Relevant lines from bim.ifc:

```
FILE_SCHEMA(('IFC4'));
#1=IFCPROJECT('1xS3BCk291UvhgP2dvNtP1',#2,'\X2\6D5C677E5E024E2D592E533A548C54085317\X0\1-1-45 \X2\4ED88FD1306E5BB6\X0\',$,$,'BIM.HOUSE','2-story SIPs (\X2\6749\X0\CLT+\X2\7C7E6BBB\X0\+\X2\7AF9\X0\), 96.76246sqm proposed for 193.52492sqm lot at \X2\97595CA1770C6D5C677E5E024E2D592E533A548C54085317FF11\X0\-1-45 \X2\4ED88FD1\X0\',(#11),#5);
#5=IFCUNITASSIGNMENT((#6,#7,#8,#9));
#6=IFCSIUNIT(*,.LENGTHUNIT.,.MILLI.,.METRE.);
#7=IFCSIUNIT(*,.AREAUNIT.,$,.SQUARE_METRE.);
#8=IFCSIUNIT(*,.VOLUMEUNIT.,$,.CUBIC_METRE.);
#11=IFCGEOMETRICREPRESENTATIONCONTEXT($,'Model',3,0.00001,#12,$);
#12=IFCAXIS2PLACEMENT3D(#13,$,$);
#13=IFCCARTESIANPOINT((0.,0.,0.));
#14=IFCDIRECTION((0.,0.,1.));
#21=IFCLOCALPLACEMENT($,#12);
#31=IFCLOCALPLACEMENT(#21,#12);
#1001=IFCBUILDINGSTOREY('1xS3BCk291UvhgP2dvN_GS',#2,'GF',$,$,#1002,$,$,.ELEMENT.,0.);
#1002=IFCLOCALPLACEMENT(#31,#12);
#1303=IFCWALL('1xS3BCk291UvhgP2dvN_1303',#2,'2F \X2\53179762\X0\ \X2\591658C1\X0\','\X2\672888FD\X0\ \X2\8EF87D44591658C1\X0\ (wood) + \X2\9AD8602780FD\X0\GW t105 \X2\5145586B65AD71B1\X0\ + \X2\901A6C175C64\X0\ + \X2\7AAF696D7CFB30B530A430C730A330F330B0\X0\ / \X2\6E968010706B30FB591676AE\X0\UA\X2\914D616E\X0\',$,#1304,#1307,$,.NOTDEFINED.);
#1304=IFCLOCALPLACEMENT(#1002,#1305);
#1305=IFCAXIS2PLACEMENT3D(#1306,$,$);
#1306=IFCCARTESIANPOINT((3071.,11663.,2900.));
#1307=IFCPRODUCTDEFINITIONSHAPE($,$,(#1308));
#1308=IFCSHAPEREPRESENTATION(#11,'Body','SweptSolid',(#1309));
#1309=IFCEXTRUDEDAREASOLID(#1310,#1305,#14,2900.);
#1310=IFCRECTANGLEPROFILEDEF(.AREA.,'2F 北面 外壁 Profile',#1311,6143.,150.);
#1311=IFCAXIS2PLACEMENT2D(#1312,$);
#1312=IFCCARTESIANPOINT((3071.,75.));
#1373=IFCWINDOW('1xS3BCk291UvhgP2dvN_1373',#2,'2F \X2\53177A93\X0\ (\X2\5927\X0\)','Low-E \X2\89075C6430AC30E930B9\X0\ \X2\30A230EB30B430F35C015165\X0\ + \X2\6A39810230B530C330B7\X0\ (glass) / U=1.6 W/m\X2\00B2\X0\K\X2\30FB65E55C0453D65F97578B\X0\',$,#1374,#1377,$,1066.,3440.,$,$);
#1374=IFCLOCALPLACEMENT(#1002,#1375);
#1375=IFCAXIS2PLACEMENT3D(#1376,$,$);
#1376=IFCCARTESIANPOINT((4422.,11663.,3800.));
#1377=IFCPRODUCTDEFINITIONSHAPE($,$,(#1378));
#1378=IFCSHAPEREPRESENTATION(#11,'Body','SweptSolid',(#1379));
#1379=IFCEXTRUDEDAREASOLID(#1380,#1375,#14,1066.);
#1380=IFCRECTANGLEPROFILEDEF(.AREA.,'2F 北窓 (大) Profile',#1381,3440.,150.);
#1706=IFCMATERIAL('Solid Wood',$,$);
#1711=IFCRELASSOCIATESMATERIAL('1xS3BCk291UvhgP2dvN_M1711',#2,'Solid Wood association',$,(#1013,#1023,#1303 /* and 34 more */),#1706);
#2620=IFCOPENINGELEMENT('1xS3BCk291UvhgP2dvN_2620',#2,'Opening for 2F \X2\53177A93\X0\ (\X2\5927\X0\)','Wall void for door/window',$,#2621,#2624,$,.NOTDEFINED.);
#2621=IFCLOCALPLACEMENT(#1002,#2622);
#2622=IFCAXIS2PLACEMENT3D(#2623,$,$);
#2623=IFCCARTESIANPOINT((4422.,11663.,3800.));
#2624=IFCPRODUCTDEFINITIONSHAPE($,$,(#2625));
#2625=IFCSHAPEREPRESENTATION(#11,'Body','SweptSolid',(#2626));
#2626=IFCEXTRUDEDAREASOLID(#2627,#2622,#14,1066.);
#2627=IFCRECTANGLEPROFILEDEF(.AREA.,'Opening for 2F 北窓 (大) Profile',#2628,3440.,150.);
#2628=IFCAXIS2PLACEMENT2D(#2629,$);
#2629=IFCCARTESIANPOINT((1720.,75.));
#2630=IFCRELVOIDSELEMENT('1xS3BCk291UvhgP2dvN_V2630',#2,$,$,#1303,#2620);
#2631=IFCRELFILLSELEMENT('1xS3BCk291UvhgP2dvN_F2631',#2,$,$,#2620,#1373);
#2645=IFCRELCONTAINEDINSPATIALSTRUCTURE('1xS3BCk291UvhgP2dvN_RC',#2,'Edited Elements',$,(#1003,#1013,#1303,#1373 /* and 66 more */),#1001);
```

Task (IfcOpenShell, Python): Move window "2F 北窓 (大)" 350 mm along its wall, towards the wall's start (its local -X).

```python
import ifcopenshell
import ifcopenshell.api.geometry
import ifcopenshell.util.placement
import ifcopenshell.util.unit

model = ifcopenshell.open("bim.ifc")
unit_scale = ifcopenshell.util.unit.calculate_unit_scale(model)

window = model.by_guid("1xS3BCk291UvhgP2dvN_1373")
opening = window.FillsVoids[0].RelatingOpeningElement
wall = opening.VoidsElements[0].RelatingBuildingElement

wall_matrix = ifcopenshell.util.placement.get_local_placement(wall.ObjectPlacement)
shift = wall_matrix[:3, 0] * -0.35 / unit_scale
before = ifcopenshell.util.placement.get_local_placement(window.ObjectPlacement)[:3, 3].copy()

# The window is not placed relative to its opening, so move both.
for product in (opening, window):
    matrix = ifcopenshell.util.placement.get_local_placement(product.ObjectPlacement)
    matrix[:3, 3] += shift
    ifcopenshell.api.geometry.edit_object_placement(model, product=product, matrix=matrix, is_si=False)

after = ifcopenshell.util.placement.get_local_placement(window.ObjectPlacement)[:3, 3]
print("window moved by", (after - before).round(3) + 0.0)

model.write("bim_v2.ifc")
```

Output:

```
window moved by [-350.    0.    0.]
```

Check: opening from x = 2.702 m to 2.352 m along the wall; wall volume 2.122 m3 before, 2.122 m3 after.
